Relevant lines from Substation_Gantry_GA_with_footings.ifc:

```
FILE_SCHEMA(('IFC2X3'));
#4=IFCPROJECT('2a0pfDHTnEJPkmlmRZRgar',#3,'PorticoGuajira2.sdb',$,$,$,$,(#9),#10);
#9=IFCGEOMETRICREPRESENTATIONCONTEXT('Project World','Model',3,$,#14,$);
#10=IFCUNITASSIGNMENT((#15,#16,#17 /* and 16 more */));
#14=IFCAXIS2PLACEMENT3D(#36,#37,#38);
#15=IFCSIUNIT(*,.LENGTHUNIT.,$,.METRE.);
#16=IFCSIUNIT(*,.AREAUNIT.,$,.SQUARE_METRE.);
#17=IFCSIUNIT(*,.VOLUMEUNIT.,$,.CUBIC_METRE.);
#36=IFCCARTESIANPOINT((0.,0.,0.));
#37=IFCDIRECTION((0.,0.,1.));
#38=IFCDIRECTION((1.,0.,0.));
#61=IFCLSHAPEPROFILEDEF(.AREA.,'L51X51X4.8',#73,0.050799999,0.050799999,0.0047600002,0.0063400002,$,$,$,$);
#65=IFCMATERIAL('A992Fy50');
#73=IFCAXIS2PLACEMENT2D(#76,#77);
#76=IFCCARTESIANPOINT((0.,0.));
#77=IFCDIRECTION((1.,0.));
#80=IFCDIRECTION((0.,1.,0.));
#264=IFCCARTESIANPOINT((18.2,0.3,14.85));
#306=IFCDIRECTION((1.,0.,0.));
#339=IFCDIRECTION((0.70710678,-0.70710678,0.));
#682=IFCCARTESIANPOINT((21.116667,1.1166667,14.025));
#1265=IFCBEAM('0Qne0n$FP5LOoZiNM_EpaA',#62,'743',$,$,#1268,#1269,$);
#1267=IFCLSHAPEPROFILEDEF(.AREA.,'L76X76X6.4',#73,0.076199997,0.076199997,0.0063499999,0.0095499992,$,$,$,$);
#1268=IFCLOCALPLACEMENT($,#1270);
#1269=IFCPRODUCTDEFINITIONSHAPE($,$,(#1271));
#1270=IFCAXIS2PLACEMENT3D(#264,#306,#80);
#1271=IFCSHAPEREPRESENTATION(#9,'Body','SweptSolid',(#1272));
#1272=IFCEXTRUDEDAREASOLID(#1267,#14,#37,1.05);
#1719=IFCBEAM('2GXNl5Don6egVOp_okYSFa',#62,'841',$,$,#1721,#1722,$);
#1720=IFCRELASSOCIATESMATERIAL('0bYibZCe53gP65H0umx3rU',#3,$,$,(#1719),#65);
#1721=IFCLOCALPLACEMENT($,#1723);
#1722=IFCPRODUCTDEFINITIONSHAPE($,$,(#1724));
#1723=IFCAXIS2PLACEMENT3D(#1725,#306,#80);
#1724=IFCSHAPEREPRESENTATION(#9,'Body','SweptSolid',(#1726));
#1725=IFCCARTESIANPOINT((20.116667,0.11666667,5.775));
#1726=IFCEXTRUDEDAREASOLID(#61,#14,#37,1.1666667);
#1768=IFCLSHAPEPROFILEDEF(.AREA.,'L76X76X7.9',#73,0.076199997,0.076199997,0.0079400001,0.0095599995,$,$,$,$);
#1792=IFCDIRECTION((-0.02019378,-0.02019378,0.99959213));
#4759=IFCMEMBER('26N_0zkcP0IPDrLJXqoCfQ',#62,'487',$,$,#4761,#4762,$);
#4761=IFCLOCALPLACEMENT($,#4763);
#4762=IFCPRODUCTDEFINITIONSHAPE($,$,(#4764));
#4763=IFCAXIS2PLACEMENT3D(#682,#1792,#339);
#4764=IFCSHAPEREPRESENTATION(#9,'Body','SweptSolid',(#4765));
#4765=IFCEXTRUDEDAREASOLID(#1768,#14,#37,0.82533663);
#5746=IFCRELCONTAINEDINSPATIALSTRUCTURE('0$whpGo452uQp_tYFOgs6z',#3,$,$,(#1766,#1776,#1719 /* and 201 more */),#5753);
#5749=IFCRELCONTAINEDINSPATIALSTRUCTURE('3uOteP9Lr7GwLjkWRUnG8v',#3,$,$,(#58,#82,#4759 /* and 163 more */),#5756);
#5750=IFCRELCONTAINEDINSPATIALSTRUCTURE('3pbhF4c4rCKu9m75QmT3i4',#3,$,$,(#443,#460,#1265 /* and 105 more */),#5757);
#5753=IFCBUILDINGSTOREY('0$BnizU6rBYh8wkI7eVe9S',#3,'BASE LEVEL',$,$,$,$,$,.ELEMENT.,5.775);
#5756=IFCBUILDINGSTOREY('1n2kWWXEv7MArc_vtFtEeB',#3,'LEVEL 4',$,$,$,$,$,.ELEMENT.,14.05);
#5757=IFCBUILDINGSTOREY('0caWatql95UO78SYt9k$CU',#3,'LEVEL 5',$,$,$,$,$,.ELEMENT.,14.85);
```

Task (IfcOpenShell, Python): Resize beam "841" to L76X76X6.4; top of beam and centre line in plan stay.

```python
import ifcopenshell
import ifcopenshell.util.element

model = ifcopenshell.open("Substation_Gantry_GA_with_footings.ifc")

member = model.by_guid("2GXNl5Don6egVOp_okYSFa")
source = next(p for p in model.by_type("IfcLShapeProfileDef") if p.ProfileName == "L76X76X6.4")

body = next(r for r in member.Representation.Representations if r.RepresentationIdentifier == "Body")
solid = body.Items[0]
old_profile = solid.SweptArea

# Copy the section's sizes but keep this member's own profile position.
profile = ifcopenshell.util.element.copy(model, source)
# Profiles are centred, so shift by half the change in depth to hold the top.
shift = (old_profile.Depth - profile.Depth) / 2
x, y = old_profile.Position.Location.Coordinates
up = (0.0, 1.0)  # upwards, in the solid's own plane
location = model.createIfcCartesianPoint((x + up[0] * shift, y + up[1] * shift))
profile.Position = model.createIfcAxis2Placement2D(location, old_profile.Position.RefDirection)
solid.SweptArea = profile
if not model.get_total_inverses(old_profile):
    ifcopenshell.util.element.remove_deep2(model, old_profile)

print(solid.SweptArea)

model.write("Substation_Gantry_GA_with_footings_edited.ifc")
```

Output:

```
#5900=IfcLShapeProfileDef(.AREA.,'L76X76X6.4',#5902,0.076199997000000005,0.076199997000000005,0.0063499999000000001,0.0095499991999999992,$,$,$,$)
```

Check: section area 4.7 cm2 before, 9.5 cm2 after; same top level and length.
